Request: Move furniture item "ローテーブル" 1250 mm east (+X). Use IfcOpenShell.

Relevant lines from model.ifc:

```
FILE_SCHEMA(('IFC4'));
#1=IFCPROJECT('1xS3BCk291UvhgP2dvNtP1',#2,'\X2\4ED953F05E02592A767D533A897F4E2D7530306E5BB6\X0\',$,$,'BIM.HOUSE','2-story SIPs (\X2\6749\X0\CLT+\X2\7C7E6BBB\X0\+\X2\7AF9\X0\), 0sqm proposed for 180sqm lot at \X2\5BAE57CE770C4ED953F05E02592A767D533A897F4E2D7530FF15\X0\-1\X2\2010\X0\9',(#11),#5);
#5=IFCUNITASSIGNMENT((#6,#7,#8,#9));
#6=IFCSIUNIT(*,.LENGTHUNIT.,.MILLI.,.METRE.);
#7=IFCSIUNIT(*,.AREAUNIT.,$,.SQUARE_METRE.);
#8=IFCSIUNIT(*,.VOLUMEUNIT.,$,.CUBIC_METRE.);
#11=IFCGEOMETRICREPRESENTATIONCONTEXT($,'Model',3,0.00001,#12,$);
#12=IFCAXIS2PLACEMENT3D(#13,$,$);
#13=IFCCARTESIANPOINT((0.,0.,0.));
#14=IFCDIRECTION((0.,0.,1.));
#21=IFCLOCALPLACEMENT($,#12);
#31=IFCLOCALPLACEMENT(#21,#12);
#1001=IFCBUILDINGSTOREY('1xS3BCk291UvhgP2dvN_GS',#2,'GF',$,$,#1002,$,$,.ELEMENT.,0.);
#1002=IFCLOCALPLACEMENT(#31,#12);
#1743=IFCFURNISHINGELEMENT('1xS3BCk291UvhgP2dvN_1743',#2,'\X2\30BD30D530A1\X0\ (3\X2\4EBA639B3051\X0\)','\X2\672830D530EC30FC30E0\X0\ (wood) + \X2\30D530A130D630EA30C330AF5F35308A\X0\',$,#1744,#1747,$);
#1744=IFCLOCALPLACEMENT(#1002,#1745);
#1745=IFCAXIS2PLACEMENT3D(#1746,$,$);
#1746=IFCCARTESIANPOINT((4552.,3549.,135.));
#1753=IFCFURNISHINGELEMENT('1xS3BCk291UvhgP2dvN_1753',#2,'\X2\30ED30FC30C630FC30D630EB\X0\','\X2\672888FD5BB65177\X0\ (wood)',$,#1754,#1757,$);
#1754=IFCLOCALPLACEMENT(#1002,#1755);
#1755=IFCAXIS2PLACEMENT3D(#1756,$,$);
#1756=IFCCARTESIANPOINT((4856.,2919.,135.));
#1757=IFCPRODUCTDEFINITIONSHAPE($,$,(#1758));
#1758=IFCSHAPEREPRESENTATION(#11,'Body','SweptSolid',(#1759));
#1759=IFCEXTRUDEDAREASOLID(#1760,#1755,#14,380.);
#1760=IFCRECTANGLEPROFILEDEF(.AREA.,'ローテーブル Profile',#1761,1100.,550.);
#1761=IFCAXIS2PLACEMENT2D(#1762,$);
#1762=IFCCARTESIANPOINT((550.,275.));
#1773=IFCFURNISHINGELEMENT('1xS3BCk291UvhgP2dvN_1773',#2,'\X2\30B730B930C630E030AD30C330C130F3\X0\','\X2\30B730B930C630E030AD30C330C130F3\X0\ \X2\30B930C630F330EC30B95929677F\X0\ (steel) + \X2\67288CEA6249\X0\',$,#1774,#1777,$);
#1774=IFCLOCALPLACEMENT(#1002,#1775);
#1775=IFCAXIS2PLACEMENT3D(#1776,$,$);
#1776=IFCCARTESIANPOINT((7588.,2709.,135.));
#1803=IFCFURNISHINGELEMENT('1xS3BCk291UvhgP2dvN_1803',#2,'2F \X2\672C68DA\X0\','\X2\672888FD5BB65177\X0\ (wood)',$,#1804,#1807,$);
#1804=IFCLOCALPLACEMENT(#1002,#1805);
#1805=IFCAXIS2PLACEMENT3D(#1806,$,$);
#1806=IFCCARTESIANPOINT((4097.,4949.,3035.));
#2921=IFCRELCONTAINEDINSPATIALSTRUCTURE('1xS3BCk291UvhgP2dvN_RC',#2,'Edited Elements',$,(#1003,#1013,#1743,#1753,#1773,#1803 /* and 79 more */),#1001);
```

```python
import ifcopenshell
import ifcopenshell.api.geometry
import ifcopenshell.util.placement

model = ifcopenshell.open("model.ifc")

item = model.by_guid("1xS3BCk291UvhgP2dvN_1753")
matrix = ifcopenshell.util.placement.get_local_placement(item.ObjectPlacement)
matrix[0, 3] += 1250.0
ifcopenshell.api.geometry.edit_object_placement(model, product=item, matrix=matrix, is_si=False)

print(ifcopenshell.util.placement.get_local_placement(item.ObjectPlacement).round(3) + 0.0)

model.write("model_rev.ifc")
```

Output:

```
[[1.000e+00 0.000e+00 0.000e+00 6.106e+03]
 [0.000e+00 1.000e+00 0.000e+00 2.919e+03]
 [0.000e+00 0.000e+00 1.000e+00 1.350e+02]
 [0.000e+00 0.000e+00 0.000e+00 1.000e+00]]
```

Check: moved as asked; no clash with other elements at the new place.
